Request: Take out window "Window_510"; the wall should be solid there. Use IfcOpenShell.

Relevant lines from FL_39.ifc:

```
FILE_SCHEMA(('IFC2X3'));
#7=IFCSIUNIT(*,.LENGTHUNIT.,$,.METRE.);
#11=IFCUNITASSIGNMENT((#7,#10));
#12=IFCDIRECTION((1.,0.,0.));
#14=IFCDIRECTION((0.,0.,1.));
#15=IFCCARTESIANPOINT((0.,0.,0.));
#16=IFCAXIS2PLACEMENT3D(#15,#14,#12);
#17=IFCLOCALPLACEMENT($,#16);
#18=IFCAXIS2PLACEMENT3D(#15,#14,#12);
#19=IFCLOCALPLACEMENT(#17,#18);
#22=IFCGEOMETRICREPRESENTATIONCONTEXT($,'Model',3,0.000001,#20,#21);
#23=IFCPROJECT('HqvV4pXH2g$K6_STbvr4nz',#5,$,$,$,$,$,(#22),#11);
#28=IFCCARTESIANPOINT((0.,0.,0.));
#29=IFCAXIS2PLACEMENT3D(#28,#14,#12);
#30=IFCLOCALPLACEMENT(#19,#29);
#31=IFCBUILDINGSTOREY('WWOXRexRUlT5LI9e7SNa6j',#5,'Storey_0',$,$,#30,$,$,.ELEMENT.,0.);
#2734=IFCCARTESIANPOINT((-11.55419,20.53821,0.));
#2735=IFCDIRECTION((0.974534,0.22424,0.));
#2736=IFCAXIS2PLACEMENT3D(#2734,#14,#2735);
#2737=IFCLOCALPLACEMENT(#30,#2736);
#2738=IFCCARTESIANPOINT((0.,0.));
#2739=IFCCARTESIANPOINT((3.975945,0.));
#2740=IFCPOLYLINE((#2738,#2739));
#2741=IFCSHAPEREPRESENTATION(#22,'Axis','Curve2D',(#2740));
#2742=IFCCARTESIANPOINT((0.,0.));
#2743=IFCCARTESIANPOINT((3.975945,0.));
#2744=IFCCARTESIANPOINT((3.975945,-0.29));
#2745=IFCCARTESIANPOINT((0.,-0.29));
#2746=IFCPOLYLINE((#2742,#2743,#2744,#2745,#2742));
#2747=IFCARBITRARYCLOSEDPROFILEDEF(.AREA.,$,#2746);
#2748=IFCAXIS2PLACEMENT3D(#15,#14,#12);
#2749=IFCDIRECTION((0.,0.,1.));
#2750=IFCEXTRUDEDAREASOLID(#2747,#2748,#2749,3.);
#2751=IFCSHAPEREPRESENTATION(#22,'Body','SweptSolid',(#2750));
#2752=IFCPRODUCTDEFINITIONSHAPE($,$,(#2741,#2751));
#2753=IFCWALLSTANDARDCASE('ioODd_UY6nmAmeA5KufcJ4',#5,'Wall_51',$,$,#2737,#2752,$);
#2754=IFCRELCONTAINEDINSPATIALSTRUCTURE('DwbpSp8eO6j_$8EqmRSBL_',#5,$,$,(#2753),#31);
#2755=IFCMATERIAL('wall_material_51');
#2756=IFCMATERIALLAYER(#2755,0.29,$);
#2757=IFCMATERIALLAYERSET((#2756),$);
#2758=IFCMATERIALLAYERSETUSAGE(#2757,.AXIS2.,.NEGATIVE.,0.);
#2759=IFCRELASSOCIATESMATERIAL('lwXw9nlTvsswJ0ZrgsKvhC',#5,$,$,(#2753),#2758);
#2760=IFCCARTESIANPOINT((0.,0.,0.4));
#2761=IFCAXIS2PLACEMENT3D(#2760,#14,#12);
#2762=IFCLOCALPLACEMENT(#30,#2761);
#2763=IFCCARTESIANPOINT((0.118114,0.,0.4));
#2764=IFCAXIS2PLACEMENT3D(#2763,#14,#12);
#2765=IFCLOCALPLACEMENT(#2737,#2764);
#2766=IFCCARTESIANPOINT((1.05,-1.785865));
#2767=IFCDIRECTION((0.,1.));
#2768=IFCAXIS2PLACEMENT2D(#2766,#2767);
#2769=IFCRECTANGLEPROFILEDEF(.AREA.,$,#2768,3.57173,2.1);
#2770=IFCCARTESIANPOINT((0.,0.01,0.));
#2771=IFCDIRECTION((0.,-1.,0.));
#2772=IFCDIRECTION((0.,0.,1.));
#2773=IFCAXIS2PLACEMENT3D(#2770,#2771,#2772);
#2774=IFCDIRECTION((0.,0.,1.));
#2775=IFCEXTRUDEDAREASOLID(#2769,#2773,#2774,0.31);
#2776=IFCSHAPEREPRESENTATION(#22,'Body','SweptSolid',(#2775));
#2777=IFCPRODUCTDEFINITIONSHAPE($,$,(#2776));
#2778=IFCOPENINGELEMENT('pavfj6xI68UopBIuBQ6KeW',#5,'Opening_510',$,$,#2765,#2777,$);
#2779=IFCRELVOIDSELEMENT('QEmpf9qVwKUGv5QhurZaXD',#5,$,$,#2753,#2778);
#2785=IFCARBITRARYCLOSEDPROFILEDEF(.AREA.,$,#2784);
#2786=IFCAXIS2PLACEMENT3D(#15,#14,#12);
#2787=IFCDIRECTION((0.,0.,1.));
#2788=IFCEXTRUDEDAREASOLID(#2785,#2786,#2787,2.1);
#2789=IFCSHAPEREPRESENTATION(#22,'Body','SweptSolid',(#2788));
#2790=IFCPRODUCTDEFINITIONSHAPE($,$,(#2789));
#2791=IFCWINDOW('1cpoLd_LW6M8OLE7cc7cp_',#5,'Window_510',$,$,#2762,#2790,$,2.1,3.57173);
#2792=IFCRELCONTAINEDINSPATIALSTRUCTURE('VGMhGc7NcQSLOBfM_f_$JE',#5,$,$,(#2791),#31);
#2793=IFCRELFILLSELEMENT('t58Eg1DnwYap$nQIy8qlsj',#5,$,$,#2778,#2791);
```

```python
import ifcopenshell
import ifcopenshell.api.feature
import ifcopenshell.api.root
import ifcopenshell.geom
import ifcopenshell.util.shape

model = ifcopenshell.open("FL_39.ifc")
settings = ifcopenshell.geom.settings()


def volume(element):
    """Net volume in cubic metres, openings subtracted."""
    shape = ifcopenshell.geom.create_shape(settings, element)
    return ifcopenshell.util.shape.get_volume(shape.geometry)


window = model.by_guid("1cpoLd_LW6M8OLE7cc7cp_")
opening = window.FillsVoids[0].RelatingOpeningElement
wall = opening.VoidsElements[0].RelatingBuildingElement
before = volume(wall)

ifcopenshell.api.root.remove_product(model, product=window)
ifcopenshell.api.feature.remove_feature(model, feature=opening)

after = volume(wall)

print(f"wall volume {before:.3f} -> {after:.3f} m3")

model.write("FL_39_updated.ifc")
```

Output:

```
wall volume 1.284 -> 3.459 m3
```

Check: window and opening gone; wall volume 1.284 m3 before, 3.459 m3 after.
